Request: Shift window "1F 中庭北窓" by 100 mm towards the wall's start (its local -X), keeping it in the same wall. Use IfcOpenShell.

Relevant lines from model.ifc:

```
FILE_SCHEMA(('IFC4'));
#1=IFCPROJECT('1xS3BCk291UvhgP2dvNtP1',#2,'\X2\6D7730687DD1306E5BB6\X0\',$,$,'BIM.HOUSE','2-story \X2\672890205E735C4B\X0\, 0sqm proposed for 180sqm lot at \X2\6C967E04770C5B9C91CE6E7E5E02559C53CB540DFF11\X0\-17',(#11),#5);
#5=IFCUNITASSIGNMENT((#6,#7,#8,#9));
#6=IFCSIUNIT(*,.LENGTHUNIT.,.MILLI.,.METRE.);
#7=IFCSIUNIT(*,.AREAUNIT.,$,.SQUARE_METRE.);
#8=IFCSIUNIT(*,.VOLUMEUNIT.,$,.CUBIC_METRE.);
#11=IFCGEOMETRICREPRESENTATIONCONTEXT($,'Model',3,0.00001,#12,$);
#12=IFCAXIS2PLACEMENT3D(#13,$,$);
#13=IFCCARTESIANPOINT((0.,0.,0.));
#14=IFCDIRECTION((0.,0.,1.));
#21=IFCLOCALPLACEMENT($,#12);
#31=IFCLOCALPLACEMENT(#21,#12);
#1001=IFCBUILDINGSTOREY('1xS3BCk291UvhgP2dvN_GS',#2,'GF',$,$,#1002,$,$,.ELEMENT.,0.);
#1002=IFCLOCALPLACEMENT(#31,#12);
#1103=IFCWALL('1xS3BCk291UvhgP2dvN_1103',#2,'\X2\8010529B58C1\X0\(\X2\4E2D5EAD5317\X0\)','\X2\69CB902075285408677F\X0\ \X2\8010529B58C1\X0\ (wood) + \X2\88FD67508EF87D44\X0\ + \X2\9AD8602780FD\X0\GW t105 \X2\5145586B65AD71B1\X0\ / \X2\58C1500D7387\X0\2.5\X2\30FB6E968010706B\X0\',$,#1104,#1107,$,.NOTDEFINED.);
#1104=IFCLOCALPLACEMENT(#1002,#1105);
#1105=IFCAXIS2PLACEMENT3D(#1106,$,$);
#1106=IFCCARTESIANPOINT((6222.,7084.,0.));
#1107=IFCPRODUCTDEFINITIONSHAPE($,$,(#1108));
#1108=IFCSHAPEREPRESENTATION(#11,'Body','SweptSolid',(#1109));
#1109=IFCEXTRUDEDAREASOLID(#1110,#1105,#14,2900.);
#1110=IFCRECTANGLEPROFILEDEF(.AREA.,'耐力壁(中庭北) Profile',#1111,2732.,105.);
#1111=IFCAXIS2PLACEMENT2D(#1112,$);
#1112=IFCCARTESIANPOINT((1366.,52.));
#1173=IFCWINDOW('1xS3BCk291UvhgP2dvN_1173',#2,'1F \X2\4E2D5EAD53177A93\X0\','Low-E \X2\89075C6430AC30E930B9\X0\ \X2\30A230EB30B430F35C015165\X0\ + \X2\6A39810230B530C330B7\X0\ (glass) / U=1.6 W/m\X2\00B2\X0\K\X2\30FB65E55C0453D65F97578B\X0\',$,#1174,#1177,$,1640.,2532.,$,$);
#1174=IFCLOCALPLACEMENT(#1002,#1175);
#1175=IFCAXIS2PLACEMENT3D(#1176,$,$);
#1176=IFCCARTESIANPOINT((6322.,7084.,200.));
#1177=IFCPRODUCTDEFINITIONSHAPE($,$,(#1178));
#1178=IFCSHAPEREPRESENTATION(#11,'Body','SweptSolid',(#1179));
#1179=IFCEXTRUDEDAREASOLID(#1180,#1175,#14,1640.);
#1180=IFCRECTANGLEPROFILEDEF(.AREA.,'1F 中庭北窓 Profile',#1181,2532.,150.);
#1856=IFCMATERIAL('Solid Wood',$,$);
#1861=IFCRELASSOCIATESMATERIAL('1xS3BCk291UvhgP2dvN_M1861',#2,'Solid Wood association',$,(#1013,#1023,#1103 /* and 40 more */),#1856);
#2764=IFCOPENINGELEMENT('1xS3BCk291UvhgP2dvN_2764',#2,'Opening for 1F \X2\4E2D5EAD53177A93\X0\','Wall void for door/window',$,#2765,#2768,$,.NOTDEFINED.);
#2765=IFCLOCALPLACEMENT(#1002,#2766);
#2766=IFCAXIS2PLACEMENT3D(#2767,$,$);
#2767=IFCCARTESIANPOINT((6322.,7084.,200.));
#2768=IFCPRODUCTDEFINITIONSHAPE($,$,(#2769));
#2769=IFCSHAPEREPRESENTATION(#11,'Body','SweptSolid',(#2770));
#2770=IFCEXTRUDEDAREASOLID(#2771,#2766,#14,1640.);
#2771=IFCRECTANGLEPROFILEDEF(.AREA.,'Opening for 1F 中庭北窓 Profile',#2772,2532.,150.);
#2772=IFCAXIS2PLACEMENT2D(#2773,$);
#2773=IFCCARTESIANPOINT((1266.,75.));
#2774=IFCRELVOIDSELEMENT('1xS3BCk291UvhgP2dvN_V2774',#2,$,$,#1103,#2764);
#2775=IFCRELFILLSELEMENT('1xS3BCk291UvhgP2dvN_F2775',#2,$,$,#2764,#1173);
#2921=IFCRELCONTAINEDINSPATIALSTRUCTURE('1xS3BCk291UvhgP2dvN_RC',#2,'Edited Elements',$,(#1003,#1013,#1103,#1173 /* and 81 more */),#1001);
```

```python
import ifcopenshell
import ifcopenshell.api.geometry
import ifcopenshell.util.placement

model = ifcopenshell.open("model.ifc")

window = model.by_guid("1xS3BCk291UvhgP2dvN_1173")
opening = window.FillsVoids[0].RelatingOpeningElement
wall = opening.VoidsElements[0].RelatingBuildingElement

wall_matrix = ifcopenshell.util.placement.get_local_placement(wall.ObjectPlacement)
shift = wall_matrix[:3, 0] * -100.0
before = ifcopenshell.util.placement.get_local_placement(window.ObjectPlacement)[:3, 3].copy()

# The window is not placed relative to its opening, so move both.
for product in (opening, window):
    matrix = ifcopenshell.util.placement.get_local_placement(product.ObjectPlacement)
    matrix[:3, 3] += shift
    ifcopenshell.api.geometry.edit_object_placement(model, product=product, matrix=matrix, is_si=False)

after = ifcopenshell.util.placement.get_local_placement(window.ObjectPlacement)[:3, 3]
print("window moved by", (after - before).round(3) + 0.0)

model.write("model_edited.ifc")
```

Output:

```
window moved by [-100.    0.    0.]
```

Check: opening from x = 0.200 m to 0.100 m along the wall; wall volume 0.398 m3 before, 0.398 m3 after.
